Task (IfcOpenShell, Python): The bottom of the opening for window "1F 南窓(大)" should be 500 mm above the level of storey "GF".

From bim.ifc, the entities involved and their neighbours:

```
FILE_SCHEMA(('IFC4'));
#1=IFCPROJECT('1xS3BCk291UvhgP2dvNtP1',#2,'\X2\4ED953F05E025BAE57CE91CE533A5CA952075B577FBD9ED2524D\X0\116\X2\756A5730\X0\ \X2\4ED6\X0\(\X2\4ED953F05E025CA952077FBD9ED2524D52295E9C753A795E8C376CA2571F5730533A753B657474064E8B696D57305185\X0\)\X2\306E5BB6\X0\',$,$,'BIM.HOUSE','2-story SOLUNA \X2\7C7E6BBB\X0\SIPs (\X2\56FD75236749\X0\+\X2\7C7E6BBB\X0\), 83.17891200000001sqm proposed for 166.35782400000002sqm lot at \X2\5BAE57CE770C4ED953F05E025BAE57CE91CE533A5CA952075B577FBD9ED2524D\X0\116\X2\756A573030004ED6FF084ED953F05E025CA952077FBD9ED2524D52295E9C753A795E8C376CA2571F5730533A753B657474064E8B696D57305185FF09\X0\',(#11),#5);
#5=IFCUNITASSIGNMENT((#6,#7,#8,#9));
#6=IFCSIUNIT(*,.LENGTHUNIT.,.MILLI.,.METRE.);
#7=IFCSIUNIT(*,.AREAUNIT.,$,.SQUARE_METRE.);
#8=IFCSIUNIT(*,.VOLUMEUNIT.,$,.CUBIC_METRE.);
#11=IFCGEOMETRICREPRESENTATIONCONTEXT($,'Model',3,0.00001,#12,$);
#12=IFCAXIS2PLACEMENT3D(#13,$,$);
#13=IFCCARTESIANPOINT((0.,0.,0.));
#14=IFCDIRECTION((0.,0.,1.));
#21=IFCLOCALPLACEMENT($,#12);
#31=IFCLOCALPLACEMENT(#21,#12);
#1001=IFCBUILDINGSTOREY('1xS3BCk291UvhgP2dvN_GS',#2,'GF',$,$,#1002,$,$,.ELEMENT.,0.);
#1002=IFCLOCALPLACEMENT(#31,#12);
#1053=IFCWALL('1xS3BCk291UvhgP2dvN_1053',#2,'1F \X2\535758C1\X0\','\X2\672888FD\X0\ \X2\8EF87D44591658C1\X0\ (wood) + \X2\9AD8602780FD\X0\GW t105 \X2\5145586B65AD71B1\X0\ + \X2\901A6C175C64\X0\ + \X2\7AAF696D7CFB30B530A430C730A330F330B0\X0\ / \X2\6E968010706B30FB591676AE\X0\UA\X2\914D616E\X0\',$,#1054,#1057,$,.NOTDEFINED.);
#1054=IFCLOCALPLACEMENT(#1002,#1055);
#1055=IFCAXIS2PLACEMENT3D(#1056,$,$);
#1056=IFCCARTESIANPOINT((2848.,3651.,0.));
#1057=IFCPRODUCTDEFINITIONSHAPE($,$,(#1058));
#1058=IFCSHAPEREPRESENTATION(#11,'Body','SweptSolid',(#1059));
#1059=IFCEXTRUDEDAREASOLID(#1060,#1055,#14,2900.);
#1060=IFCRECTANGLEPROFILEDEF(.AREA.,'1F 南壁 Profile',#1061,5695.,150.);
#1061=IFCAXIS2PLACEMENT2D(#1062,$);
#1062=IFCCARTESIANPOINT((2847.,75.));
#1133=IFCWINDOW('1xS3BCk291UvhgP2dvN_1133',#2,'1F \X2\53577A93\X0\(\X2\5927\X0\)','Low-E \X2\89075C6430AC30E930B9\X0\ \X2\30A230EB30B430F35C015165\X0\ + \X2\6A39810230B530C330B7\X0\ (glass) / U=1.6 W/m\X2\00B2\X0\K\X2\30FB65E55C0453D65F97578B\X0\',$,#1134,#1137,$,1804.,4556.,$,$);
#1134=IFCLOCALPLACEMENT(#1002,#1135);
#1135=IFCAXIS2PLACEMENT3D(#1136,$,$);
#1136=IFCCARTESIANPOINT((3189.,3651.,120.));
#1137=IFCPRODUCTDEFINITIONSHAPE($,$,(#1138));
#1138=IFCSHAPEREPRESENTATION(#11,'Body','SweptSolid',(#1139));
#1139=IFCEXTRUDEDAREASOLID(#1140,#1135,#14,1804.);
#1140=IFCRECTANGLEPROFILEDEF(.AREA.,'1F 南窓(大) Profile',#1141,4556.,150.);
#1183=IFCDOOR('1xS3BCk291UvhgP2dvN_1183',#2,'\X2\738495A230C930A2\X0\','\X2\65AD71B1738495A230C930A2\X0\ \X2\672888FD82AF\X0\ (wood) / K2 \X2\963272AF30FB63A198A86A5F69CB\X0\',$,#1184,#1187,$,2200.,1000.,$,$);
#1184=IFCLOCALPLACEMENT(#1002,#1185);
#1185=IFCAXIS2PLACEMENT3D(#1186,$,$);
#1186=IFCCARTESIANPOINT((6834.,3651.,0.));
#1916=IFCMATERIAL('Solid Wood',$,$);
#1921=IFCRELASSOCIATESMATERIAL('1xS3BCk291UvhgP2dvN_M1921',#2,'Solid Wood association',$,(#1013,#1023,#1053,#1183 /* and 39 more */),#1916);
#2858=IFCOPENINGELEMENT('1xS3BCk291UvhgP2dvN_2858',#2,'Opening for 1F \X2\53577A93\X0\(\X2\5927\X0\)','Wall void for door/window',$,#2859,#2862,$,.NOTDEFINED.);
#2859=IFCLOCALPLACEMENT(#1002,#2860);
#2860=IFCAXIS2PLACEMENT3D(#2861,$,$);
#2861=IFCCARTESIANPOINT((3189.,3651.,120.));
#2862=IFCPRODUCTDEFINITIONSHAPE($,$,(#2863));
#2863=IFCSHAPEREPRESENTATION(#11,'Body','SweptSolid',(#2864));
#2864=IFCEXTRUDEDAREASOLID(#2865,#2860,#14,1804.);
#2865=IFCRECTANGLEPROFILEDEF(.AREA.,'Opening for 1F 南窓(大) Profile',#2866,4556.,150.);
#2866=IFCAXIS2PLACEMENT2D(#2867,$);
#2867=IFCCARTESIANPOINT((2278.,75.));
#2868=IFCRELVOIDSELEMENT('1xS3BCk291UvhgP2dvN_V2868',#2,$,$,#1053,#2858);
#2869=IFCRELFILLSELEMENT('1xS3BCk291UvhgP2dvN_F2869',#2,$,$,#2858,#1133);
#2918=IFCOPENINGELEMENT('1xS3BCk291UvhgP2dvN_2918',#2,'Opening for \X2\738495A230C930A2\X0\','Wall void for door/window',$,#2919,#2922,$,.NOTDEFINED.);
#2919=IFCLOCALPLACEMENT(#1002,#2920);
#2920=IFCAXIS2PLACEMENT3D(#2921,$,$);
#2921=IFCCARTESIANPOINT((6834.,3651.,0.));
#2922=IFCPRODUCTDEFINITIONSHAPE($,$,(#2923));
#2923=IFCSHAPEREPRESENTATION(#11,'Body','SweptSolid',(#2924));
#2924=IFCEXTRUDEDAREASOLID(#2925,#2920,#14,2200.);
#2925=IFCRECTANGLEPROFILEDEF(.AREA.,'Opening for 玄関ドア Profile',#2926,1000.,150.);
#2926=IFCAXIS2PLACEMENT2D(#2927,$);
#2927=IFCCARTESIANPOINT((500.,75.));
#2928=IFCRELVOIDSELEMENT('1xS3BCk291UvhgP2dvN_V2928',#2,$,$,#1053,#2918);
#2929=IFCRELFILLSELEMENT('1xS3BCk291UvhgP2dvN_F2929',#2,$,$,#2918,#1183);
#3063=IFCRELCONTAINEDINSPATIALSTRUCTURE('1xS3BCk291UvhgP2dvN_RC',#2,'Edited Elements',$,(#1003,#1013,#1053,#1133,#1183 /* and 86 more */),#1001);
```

```python
import numpy as np
import ifcopenshell
import ifcopenshell.api.geometry
import ifcopenshell.geom
import ifcopenshell.util.element
import ifcopenshell.util.placement
import ifcopenshell.util.shape
import ifcopenshell.util.unit

model = ifcopenshell.open("bim.ifc")
unit_scale = ifcopenshell.util.unit.calculate_unit_scale(model)

window = model.by_id(1133)
opening = window.FillsVoids[0].RelatingOpeningElement
storey = ifcopenshell.util.element.get_container(window, ifc_class="IfcBuildingStorey")
level = ifcopenshell.util.placement.get_local_placement(storey.ObjectPlacement)[2, 3]

# The opening's origin need not be at the sill, so measure its lowest point.
shape = ifcopenshell.geom.create_shape(ifcopenshell.geom.settings(), opening)
bottom = ifcopenshell.util.shape.get_shape_bottom_elevation(shape, shape.geometry) / unit_scale
dz = level + 0.5 / unit_scale - bottom

shift = np.array([0.0, 0.0, dz])
# The window is not placed relative to its opening, so move both.
for product in (opening, window):
    matrix = ifcopenshell.util.placement.get_local_placement(product.ObjectPlacement)
    matrix[:3, 3] += shift
    ifcopenshell.api.geometry.edit_object_placement(model, product=product, matrix=matrix, is_si=False)

print(f"moved by {dz * unit_scale:+.3f} m")

model.write("bim_rev.ifc")
```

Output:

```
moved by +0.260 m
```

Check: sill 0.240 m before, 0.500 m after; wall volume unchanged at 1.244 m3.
